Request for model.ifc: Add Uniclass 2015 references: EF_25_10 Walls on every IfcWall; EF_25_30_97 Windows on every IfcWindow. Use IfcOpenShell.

First a look at what the model holds.

```python
import ifcopenshell

model = ifcopenshell.open("model.ifc")
print(model.schema)
print("classifications:", [c.Name for c in model.by_type("IfcClassification")])
for ifc_class in ("IfcDoor", "IfcRoof", "IfcStair", "IfcWall", "IfcWindow"):
    print(ifc_class, len(model.by_type(ifc_class)))
```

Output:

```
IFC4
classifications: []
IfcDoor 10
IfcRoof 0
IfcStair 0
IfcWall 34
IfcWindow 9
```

```python
import ifcopenshell
import ifcopenshell.api.classification

model = ifcopenshell.open("model.ifc")

system = ifcopenshell.api.classification.add_classification(model, classification="Uniclass 2015")

codes = {
    "IfcWall": ("EF_25_10", "Walls"),
    "IfcWindow": ("EF_25_30_97", "Windows"),
}
for ifc_class, (code, name) in codes.items():
    products = model.by_type(ifc_class)
    ifcopenshell.api.classification.add_reference(
        model, products=products, classification=system, identification=code, name=name
    )
    print(code, len(products))

model.write("model-out.ifc")
```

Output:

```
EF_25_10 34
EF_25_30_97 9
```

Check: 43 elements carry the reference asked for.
